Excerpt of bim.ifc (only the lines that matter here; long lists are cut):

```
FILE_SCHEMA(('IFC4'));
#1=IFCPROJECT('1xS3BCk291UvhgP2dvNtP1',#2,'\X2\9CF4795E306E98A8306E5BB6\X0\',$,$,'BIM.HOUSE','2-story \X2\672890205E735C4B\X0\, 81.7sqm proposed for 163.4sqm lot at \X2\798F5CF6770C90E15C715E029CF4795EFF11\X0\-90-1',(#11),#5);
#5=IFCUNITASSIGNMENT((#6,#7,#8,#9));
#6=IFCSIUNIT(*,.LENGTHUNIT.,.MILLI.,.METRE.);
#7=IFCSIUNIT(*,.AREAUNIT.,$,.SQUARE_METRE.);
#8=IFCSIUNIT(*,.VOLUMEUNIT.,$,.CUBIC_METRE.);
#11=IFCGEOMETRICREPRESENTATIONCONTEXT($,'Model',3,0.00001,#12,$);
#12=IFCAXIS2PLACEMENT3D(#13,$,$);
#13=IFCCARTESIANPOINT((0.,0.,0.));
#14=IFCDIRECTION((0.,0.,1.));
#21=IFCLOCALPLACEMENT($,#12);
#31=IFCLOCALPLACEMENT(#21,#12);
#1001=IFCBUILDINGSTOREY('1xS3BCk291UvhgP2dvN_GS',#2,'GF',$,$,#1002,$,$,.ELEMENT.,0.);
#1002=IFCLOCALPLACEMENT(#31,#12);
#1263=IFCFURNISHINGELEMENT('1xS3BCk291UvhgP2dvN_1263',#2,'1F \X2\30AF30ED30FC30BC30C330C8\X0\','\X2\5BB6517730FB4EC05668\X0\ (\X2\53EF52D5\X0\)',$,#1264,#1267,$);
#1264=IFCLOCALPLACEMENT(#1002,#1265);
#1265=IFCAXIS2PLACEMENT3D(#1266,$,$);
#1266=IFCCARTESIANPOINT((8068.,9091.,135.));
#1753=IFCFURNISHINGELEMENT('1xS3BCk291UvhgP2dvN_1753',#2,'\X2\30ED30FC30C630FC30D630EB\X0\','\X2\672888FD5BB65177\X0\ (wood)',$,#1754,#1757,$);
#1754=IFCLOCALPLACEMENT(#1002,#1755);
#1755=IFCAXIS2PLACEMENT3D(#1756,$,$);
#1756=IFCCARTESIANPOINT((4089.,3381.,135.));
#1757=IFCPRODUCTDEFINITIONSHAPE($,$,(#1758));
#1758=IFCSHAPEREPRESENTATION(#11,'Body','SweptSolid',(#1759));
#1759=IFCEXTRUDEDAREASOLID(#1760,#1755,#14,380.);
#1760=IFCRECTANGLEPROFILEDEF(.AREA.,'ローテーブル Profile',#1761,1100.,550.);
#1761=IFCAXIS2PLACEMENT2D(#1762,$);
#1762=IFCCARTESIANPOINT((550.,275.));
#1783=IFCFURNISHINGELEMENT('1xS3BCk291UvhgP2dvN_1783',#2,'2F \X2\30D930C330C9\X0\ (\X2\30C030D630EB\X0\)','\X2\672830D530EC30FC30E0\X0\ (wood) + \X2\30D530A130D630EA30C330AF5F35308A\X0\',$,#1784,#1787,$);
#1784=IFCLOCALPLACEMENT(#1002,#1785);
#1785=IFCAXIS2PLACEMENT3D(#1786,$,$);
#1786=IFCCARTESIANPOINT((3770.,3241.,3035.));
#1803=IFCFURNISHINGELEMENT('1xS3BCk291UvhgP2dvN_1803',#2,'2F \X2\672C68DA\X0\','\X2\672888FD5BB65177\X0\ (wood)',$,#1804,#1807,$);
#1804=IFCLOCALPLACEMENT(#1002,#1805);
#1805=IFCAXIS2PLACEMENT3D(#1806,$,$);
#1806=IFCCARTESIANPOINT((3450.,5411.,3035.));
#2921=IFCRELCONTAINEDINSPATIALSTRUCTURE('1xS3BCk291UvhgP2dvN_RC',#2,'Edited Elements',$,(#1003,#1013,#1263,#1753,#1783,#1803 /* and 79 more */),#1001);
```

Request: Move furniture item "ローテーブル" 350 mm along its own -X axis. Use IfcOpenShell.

```python
import ifcopenshell
import ifcopenshell.api.geometry
import ifcopenshell.util.placement
import ifcopenshell.util.unit

model = ifcopenshell.open("bim.ifc")
unit_scale = ifcopenshell.util.unit.calculate_unit_scale(model)

item = model.by_id(1753)
matrix = ifcopenshell.util.placement.get_local_placement(item.ObjectPlacement)
matrix[:3, 3] -= matrix[:3, 0] * 0.35 / unit_scale
ifcopenshell.api.geometry.edit_object_placement(model, product=item, matrix=matrix, is_si=False)

print(ifcopenshell.util.placement.get_local_placement(item.ObjectPlacement).round(3) + 0.0)

model.write("bim-out.ifc")
```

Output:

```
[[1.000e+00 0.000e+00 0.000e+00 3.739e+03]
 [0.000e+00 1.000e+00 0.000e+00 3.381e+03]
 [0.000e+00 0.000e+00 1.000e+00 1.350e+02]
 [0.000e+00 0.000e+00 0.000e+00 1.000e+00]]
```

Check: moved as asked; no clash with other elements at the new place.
